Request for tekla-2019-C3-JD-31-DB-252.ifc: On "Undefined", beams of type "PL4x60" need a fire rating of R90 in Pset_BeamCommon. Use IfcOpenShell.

First a look at what the model holds.

```python
import ifcopenshell
import ifcopenshell.util.element

model = ifcopenshell.open("tekla-2019-C3-JD-31-DB-252.ifc")
print(model.schema)
storey = next(s for s in model.by_type("IfcBuildingStorey") if s.Name == "Undefined")
beams = [e for e in ifcopenshell.util.element.get_decomposition(storey) if e.is_a("IfcBeam")]
seen = {}
for e in beams:
    element_type = ifcopenshell.util.element.get_type(e)
    key = (element_type.Name if element_type != e and element_type else None, ifcopenshell.util.element.get_pset(e, "Pset_BeamCommon", "FireRating"))
    seen[key] = seen.get(key, 0) + 1
for (name, value), count in sorted(seen.items(), key=str):
    print(count, "x", name, "|", value)
```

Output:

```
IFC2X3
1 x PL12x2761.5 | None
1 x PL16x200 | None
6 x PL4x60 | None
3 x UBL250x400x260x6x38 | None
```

```python
import ifcopenshell
import ifcopenshell.api.pset
import ifcopenshell.util.element

model = ifcopenshell.open("tekla-2019-C3-JD-31-DB-252.ifc")

storey = next(s for s in model.by_type("IfcBuildingStorey") if s.Name == "Undefined")
beams = [e for e in ifcopenshell.util.element.get_decomposition(storey) if e.is_a("IfcBeam")]

count = 0
for e in beams:
    element_type = ifcopenshell.util.element.get_type(e)
    if element_type in (None, e) or element_type.Name != "PL4x60":
        continue
    found = ifcopenshell.util.element.get_pset(e, "Pset_BeamCommon", should_inherit=False)
    if found:
        pset = model.by_id(found["id"])
        if len(ifcopenshell.util.element.get_elements_by_pset(pset)) > 1:
            pset = ifcopenshell.api.pset.unshare_pset(model, products=[e], pset=pset)[0]
    else:
        pset = ifcopenshell.api.pset.add_pset(model, product=e, name="Pset_BeamCommon")
    ifcopenshell.api.pset.edit_pset(model, pset=pset, properties={"FireRating": "R90"})
    count += 1

print(count, "beams updated")

model.write("tekla-2019-C3-JD-31-DB-252_v2.ifc")
```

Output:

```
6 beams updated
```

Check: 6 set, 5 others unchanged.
